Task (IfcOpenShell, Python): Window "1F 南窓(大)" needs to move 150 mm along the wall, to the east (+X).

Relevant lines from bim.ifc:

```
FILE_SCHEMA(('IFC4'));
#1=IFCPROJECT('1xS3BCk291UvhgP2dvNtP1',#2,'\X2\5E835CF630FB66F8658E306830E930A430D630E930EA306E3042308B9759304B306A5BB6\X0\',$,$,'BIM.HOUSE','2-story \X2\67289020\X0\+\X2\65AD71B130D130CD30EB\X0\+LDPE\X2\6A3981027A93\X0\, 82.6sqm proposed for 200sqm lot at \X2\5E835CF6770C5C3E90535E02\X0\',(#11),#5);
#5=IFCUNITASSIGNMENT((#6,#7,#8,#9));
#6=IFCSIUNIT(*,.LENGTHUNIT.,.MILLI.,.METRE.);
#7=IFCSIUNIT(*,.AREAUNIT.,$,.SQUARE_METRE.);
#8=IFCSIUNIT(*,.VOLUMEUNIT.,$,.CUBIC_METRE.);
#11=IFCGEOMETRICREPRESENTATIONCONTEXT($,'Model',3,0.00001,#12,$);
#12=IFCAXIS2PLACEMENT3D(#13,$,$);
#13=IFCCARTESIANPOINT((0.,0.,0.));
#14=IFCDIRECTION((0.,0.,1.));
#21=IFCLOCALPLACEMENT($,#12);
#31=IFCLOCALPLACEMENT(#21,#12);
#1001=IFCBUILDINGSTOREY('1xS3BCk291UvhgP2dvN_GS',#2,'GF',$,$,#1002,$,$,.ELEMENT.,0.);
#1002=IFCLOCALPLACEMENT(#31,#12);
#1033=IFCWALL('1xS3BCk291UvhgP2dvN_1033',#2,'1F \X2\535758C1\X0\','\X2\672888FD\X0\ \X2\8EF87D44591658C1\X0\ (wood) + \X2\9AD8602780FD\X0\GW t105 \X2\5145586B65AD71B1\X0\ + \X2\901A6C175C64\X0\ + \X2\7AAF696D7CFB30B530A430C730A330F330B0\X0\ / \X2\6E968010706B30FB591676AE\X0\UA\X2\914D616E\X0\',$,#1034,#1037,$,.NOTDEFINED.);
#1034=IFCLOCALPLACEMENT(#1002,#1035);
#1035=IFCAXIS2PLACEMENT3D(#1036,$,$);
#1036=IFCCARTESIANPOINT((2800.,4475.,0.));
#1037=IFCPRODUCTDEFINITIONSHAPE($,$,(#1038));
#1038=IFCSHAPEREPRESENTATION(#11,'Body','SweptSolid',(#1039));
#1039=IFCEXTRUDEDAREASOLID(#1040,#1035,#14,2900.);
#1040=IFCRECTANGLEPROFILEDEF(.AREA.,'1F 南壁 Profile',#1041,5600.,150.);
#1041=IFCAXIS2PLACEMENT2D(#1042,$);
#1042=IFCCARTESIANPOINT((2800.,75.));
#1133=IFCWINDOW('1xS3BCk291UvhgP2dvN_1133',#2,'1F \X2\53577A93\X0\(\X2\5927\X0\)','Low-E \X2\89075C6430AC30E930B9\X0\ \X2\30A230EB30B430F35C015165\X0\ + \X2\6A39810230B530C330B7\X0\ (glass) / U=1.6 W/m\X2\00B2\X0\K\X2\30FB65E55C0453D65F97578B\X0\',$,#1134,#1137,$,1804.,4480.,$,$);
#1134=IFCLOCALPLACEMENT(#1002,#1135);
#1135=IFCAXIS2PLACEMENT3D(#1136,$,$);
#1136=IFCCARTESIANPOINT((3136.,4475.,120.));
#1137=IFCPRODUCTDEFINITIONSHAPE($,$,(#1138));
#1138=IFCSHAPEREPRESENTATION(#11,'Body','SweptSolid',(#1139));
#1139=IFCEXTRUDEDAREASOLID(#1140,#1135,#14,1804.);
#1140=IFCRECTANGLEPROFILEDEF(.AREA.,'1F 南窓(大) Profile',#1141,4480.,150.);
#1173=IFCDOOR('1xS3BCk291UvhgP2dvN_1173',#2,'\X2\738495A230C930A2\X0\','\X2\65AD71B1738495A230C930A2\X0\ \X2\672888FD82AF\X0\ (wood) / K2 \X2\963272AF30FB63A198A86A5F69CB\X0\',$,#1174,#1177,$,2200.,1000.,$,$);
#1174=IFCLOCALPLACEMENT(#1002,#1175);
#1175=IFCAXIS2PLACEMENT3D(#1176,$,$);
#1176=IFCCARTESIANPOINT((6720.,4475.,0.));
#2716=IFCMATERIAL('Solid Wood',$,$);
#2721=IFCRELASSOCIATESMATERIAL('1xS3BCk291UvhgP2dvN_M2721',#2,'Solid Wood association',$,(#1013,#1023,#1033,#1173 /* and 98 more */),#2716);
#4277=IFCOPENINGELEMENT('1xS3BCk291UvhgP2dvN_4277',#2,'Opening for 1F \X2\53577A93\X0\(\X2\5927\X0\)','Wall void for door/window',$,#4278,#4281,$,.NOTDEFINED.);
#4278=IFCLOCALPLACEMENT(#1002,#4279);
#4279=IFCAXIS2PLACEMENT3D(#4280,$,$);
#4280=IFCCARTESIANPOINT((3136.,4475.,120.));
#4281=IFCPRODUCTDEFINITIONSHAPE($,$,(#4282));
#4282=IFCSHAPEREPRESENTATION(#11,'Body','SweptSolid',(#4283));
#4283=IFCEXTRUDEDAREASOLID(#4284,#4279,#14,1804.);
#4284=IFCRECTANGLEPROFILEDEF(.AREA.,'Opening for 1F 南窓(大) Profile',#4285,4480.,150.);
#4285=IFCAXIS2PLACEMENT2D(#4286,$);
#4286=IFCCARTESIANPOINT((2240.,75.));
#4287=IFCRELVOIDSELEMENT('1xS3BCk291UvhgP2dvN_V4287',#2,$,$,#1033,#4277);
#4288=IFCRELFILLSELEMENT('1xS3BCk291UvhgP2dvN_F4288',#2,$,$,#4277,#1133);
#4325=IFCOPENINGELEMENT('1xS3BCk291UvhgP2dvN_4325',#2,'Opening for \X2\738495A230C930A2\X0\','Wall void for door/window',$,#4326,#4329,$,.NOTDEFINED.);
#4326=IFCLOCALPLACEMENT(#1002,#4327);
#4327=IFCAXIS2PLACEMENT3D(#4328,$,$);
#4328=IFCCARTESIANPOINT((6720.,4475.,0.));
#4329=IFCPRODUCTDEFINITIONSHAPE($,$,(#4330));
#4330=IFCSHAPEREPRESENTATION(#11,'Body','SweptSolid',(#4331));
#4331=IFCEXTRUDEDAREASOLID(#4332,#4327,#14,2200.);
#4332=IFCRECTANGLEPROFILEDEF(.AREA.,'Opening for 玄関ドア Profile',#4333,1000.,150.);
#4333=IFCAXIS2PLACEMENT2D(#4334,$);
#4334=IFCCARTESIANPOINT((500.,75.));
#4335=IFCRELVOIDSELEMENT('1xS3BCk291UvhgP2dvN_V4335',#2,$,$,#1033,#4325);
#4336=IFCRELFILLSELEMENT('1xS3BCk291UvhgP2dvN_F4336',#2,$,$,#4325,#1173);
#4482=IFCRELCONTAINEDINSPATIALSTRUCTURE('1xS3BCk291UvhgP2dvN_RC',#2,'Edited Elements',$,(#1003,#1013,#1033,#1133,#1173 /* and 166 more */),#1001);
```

```python
import ifcopenshell
import ifcopenshell.api.geometry
import ifcopenshell.util.placement

model = ifcopenshell.open("bim.ifc")

window = model.by_id(1133)
opening = window.FillsVoids[0].RelatingOpeningElement
wall = opening.VoidsElements[0].RelatingBuildingElement

wall_matrix = ifcopenshell.util.placement.get_local_placement(wall.ObjectPlacement)
shift = wall_matrix[:3, 0] * 150.0
before = ifcopenshell.util.placement.get_local_placement(window.ObjectPlacement)[:3, 3].copy()

# The window is not placed relative to its opening, so move both.
for product in (opening, window):
    matrix = ifcopenshell.util.placement.get_local_placement(product.ObjectPlacement)
    matrix[:3, 3] += shift
    ifcopenshell.api.geometry.edit_object_placement(model, product=product, matrix=matrix, is_si=False)

after = ifcopenshell.util.placement.get_local_placement(window.ObjectPlacement)[:3, 3]
print("window moved by", (after - before).round(3) + 0.0)

model.write("bim_updated.ifc")
```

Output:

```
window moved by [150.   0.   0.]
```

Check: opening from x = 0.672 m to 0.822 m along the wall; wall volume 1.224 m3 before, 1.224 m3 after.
